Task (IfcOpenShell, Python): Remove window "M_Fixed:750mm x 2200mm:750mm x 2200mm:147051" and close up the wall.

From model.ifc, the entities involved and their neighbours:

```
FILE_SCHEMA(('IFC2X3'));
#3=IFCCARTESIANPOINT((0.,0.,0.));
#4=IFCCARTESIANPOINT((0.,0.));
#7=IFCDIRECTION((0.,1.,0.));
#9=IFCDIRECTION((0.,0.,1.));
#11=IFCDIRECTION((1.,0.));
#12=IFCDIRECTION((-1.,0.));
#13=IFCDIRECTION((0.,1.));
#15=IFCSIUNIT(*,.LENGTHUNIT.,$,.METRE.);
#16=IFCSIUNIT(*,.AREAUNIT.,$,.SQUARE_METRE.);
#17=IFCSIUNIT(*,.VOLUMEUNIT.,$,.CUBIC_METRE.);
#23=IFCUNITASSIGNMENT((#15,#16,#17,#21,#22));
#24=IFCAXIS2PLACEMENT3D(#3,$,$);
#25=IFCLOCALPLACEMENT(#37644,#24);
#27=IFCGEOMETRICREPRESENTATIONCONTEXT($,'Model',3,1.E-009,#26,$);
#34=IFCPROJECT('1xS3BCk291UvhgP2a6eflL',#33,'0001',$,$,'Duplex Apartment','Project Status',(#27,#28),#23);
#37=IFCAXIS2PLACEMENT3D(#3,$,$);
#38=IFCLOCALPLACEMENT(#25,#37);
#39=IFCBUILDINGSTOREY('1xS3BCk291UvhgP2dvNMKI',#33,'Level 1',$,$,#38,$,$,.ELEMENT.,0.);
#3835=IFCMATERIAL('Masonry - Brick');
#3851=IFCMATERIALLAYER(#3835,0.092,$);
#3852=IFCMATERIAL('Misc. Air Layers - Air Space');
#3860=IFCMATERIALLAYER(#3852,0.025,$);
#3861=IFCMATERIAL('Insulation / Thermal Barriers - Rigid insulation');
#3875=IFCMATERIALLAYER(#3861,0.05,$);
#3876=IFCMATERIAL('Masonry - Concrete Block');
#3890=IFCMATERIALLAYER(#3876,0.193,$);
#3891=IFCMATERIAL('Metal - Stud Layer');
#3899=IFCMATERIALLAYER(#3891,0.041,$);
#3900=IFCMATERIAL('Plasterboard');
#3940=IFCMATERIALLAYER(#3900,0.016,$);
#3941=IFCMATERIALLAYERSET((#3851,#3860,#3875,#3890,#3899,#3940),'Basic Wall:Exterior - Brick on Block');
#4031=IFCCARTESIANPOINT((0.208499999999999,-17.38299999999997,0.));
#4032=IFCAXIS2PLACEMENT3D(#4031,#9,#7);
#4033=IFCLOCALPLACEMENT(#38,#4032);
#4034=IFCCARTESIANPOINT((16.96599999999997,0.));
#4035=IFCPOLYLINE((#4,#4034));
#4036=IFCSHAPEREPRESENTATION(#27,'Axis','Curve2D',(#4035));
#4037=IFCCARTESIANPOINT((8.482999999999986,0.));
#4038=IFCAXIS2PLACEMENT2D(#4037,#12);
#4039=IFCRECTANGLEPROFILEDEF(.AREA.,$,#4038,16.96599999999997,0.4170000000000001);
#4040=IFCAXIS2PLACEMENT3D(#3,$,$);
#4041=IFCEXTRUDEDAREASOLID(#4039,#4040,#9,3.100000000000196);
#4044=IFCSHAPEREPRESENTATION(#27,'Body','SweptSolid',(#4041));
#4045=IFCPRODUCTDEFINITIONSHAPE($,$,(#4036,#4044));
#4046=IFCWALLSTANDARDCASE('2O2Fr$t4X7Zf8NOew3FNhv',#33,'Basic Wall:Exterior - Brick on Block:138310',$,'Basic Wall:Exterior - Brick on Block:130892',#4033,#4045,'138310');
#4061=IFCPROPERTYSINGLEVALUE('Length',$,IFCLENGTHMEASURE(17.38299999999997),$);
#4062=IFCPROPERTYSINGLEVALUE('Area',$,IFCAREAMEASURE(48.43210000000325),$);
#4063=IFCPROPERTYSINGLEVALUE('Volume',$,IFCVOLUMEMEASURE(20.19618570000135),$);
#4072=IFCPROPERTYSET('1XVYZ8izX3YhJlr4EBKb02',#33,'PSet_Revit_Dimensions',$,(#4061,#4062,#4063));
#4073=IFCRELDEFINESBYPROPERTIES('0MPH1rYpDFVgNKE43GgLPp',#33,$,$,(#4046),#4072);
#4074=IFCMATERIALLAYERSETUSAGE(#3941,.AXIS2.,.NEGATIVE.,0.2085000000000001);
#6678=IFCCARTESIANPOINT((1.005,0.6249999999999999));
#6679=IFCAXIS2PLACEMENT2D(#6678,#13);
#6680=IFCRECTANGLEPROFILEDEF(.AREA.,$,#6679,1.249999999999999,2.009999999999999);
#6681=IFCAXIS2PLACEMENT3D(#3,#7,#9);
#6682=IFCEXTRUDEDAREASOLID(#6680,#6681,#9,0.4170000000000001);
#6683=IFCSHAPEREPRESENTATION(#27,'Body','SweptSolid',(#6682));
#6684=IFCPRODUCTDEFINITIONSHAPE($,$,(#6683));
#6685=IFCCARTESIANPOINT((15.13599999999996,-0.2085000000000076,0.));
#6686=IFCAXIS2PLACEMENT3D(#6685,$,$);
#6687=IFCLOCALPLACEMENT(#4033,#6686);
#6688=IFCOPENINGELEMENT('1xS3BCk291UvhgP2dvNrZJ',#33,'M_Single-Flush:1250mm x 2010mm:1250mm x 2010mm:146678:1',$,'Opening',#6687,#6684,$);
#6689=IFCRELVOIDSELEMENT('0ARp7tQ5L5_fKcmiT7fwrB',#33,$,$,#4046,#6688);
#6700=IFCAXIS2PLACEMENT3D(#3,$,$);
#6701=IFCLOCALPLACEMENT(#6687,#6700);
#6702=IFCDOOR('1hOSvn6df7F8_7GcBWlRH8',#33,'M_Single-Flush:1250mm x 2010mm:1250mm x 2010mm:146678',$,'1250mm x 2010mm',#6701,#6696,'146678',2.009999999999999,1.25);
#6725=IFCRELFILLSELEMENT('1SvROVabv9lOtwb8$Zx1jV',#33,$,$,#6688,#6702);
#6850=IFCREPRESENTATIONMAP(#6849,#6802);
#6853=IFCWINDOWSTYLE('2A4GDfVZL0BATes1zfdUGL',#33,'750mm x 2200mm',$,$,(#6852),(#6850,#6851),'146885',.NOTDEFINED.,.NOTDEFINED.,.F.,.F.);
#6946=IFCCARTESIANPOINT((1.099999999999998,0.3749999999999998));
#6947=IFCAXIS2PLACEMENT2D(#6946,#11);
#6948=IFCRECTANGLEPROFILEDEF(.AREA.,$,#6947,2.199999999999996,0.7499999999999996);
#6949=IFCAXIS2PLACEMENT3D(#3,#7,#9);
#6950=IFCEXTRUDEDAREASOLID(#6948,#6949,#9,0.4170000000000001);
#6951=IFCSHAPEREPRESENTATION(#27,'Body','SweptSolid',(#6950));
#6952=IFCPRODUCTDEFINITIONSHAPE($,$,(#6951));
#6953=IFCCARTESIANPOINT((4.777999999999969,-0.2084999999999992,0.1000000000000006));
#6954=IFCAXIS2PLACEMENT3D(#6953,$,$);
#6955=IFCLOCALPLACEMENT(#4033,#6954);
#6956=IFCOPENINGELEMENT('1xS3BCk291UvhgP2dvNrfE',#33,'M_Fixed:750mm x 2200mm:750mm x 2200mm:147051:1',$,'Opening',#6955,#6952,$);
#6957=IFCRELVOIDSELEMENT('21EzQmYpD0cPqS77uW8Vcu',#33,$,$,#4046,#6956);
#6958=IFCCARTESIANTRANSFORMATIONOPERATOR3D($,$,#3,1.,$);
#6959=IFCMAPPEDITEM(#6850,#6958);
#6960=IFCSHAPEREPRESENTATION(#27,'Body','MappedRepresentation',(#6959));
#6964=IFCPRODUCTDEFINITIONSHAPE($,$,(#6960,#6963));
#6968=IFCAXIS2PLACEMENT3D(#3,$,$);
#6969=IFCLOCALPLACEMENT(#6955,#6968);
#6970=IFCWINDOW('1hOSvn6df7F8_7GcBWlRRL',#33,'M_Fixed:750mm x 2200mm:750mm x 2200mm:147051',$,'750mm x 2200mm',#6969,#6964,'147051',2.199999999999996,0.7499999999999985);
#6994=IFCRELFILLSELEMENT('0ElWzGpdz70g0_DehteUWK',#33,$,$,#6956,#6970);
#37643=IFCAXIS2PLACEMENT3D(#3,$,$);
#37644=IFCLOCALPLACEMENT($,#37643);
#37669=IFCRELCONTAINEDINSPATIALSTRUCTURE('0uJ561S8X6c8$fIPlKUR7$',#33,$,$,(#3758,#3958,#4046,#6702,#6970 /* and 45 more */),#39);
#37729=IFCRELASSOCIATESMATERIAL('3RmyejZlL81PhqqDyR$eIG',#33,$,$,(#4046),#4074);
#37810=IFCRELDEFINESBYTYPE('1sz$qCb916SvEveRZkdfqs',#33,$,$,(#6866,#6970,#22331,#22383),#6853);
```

```python
import ifcopenshell
import ifcopenshell.api.feature
import ifcopenshell.api.pset
import ifcopenshell.api.root
import ifcopenshell.geom
import ifcopenshell.util.element
import ifcopenshell.util.shape
import ifcopenshell.util.unit

model = ifcopenshell.open("model.ifc")
area_scale = ifcopenshell.util.unit.calculate_unit_scale(model, "AREAUNIT")
volume_scale = ifcopenshell.util.unit.calculate_unit_scale(model, "VOLUMEUNIT")
settings = ifcopenshell.geom.settings()


def volume(element):
    """Net volume in cubic metres, openings subtracted."""
    shape = ifcopenshell.geom.create_shape(settings, element)
    return ifcopenshell.util.shape.get_volume(shape.geometry)


window = model.by_guid("1hOSvn6df7F8_7GcBWlRRL")
opening = window.FillsVoids[0].RelatingOpeningElement
wall = opening.VoidsElements[0].RelatingBuildingElement
before = volume(wall)

ifcopenshell.api.root.remove_product(model, product=window)
ifcopenshell.api.feature.remove_feature(model, feature=opening)

after = volume(wall)
thickness = 0.417  # wall thickness in metres

# Update the wall's stored quantities.
pset = model.by_id(ifcopenshell.util.element.get_pset(wall, "PSet_Revit_Dimensions", should_inherit=False)["id"])
ifcopenshell.api.pset.edit_pset(model, pset=pset, properties={
    "Area": model.create_entity("IfcAreaMeasure", after / thickness / area_scale),
    "Volume": model.create_entity("IfcVolumeMeasure", after / volume_scale),
})

print(f"wall volume {before:.3f} -> {after:.3f} m3")

model.write("model_v2.ifc")
```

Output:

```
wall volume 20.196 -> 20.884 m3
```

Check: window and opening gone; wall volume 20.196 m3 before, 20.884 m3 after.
